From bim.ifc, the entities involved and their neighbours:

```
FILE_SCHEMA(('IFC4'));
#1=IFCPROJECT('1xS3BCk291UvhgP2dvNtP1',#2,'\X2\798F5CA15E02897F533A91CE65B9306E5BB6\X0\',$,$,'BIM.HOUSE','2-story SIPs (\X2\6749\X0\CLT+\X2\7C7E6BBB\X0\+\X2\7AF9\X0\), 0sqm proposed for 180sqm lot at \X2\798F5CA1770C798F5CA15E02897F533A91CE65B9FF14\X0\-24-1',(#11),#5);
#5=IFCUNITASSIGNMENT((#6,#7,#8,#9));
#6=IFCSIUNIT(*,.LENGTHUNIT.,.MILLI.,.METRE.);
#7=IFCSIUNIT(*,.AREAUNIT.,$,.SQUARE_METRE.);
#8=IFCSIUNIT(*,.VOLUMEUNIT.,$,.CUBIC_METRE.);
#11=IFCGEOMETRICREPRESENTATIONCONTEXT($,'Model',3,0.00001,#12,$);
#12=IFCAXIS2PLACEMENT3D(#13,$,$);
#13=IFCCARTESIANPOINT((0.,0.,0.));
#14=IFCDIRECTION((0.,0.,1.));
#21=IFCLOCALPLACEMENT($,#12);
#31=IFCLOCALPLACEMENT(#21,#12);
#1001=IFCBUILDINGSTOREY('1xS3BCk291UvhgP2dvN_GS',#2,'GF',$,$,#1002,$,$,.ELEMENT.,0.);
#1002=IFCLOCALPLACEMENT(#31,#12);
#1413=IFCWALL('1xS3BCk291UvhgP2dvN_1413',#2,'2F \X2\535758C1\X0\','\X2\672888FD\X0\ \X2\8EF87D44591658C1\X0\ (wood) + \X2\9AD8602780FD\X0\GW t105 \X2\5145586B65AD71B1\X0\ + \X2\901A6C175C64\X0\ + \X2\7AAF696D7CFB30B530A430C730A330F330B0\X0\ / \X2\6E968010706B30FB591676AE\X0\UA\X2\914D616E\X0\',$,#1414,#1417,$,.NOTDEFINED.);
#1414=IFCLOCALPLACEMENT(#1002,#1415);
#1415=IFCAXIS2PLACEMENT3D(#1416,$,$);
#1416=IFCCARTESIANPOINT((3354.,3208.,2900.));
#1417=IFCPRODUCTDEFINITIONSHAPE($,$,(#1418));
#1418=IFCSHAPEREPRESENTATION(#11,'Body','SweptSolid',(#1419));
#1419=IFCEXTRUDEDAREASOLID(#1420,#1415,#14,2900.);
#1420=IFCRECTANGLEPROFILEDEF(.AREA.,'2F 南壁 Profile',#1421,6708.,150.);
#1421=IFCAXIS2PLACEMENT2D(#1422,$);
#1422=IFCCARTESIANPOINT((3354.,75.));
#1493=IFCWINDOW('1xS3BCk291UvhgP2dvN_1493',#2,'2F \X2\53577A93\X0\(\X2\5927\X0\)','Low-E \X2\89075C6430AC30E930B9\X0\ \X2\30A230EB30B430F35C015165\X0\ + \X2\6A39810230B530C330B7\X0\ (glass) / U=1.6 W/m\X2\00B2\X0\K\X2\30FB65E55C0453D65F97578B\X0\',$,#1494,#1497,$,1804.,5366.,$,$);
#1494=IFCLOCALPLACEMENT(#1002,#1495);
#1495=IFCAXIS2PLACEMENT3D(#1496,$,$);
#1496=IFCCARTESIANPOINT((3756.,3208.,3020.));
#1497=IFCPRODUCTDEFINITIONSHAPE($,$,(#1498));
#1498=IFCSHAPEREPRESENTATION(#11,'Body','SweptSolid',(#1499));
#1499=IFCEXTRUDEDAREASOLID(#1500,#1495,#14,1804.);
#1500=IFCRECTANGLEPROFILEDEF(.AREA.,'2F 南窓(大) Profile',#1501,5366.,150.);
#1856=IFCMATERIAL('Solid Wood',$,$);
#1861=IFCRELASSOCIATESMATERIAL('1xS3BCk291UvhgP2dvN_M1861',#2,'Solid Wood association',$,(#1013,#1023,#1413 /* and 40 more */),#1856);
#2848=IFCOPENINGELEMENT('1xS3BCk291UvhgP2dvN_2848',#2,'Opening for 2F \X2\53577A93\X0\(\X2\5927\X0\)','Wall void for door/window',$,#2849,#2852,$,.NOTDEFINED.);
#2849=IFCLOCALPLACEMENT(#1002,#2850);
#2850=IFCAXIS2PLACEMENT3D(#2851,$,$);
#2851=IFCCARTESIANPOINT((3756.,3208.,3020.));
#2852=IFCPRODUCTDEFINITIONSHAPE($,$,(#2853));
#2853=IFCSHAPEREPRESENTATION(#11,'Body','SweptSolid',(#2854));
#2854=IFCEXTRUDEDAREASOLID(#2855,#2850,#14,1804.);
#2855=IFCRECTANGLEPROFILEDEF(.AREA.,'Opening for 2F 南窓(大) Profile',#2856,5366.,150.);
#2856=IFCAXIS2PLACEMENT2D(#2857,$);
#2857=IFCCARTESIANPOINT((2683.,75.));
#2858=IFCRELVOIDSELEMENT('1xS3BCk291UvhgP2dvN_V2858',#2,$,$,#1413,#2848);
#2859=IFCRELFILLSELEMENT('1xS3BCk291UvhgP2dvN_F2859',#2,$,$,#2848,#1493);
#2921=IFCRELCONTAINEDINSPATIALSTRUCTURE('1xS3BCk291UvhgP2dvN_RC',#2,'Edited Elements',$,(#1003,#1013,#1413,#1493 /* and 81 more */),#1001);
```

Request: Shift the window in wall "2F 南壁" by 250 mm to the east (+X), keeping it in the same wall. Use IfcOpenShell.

```python
import ifcopenshell
import ifcopenshell.api.geometry
import ifcopenshell.util.placement
import ifcopenshell.util.unit

model = ifcopenshell.open("bim.ifc")
unit_scale = ifcopenshell.util.unit.calculate_unit_scale(model)

window = model.by_guid("1xS3BCk291UvhgP2dvN_1493")
opening = window.FillsVoids[0].RelatingOpeningElement
wall = opening.VoidsElements[0].RelatingBuildingElement

wall_matrix = ifcopenshell.util.placement.get_local_placement(wall.ObjectPlacement)
shift = wall_matrix[:3, 0] * 0.25 / unit_scale
before = ifcopenshell.util.placement.get_local_placement(window.ObjectPlacement)[:3, 3].copy()

# The window is not placed relative to its opening, so move both.
for product in (opening, window):
    matrix = ifcopenshell.util.placement.get_local_placement(product.ObjectPlacement)
    matrix[:3, 3] += shift
    ifcopenshell.api.geometry.edit_object_placement(model, product=product, matrix=matrix, is_si=False)

after = ifcopenshell.util.placement.get_local_placement(window.ObjectPlacement)[:3, 3]
print("window moved by", (after - before).round(3) + 0.0)

model.write("bim_edited.ifc")
```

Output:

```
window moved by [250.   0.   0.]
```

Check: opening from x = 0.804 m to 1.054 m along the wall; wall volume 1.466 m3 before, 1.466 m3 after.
